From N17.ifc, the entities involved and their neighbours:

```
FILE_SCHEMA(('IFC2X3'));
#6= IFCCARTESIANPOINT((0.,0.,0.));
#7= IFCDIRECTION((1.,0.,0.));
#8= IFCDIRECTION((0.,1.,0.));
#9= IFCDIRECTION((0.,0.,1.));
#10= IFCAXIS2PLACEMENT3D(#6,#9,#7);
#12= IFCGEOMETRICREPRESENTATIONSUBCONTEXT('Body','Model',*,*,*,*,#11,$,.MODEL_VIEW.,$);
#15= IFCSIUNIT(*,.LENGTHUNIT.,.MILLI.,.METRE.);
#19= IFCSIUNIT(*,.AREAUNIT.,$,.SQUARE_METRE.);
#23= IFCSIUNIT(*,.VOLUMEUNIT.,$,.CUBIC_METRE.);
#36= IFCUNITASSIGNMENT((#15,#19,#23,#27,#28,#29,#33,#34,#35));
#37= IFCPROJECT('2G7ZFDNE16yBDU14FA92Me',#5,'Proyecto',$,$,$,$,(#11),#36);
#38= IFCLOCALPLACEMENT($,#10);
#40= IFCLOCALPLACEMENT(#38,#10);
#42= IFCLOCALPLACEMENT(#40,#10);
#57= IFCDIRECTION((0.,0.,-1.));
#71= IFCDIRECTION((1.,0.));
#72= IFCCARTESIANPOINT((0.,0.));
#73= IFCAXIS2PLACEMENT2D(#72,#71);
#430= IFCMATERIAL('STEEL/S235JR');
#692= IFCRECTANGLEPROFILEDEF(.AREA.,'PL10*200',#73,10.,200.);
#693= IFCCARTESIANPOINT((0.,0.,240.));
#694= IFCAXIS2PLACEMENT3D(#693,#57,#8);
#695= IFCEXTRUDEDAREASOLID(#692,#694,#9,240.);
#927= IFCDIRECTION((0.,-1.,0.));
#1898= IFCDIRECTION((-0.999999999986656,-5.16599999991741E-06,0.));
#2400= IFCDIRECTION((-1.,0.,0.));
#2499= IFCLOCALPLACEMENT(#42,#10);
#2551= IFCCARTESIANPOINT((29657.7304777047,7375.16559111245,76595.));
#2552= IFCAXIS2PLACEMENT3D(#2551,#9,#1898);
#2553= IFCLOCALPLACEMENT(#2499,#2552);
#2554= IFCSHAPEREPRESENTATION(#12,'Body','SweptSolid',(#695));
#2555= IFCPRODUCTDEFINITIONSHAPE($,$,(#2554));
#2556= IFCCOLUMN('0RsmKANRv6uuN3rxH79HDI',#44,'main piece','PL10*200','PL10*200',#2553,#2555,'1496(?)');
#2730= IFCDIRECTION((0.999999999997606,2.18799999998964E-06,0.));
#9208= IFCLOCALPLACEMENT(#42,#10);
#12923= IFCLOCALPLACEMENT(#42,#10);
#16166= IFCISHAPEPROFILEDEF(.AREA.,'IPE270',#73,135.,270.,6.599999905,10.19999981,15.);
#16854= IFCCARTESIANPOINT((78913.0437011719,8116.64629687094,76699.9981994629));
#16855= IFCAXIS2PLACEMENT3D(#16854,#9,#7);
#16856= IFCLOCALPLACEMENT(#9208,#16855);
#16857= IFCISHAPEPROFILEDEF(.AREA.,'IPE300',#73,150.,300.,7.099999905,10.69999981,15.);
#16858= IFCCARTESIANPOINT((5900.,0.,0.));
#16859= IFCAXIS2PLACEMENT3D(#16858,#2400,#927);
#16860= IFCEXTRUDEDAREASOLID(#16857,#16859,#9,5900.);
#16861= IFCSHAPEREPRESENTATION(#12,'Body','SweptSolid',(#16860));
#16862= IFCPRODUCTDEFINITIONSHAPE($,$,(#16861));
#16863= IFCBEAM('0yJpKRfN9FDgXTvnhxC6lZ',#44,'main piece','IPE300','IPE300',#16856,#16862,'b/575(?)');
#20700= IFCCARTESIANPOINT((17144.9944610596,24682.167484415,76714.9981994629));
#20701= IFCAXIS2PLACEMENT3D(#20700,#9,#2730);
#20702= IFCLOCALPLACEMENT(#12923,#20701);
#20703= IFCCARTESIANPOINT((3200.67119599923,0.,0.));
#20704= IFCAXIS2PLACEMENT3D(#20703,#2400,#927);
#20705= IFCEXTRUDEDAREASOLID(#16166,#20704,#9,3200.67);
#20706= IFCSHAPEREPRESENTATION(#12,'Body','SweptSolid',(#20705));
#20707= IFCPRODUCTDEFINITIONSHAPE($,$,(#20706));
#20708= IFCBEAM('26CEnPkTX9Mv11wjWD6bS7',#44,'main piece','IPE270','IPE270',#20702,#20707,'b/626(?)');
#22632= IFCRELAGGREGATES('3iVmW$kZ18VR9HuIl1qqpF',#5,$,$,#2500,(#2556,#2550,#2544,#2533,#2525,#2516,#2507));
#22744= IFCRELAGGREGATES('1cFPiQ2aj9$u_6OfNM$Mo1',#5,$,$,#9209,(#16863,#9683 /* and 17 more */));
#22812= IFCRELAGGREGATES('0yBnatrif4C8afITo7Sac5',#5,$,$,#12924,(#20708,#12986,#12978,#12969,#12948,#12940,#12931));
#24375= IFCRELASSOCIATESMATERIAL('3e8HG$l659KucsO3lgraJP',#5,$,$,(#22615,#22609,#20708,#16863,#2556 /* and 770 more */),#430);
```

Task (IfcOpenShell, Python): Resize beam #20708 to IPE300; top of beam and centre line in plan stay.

```python
import ifcopenshell
import ifcopenshell.util.element
import ifcopenshell.util.representation

model = ifcopenshell.open("N17.ifc")

member = model.by_guid("26CEnPkTX9Mv11wjWD6bS7")
source = next(p for p in model.by_type("IfcIShapeProfileDef") if p.ProfileName == "IPE300")

body = ifcopenshell.util.representation.get_representation(member, "Model", "Body")
solid = body.Items[0]
old_profile = solid.SweptArea

# Copy the section's sizes but keep this member's own profile position.
profile = ifcopenshell.util.element.copy(model, source)
# Profiles are centred, so shift by half the change in depth to hold the top.
shift = (old_profile.OverallDepth - profile.OverallDepth) / 2
x, y = old_profile.Position.Location.Coordinates
up = (0.0, 1.0)  # upwards, in the solid's own plane
location = model.createIfcCartesianPoint((x + up[0] * shift, y + up[1] * shift))
profile.Position = model.createIfcAxis2Placement2D(location, old_profile.Position.RefDirection)
solid.SweptArea = profile
if not model.get_total_inverses(old_profile):
    ifcopenshell.util.element.remove_deep2(model, old_profile)
member.Description = member.Description.replace("IPE270", "IPE300")
member.ObjectType = member.ObjectType.replace("IPE270", "IPE300")

print(solid.SweptArea)

model.write("N17-out.ifc")
```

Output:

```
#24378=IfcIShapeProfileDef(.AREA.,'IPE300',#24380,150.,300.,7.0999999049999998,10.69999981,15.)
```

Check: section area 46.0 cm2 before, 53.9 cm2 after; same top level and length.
